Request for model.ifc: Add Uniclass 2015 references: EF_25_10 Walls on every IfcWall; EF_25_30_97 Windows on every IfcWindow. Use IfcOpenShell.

First a look at what the model holds.

```python
import ifcopenshell

model = ifcopenshell.open("model.ifc")
print(model.schema)
print("classifications:", [c.Name for c in model.by_type("IfcClassification")])
for ifc_class in ("IfcDoor", "IfcRoof", "IfcStair", "IfcWall", "IfcWindow"):
    print(ifc_class, len(model.by_type(ifc_class)))
```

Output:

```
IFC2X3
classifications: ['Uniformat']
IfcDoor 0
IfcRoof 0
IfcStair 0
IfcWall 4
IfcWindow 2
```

```python
import ifcopenshell
import ifcopenshell.api.classification

model = ifcopenshell.open("model.ifc")

# IFC2X3 requires Source and Edition and has no link from the project to the system.
system = model.create_entity("IfcClassification", Source="NBS", Edition="2015", Name="Uniclass 2015")

codes = {
    "IfcWall": ("EF_25_10", "Walls"),
    "IfcWindow": ("EF_25_30_97", "Windows"),
}
for ifc_class, (code, name) in codes.items():
    products = model.by_type(ifc_class)
    ifcopenshell.api.classification.add_reference(
        model, products=products, classification=system, identification=code, name=name
    )
    print(code, len(products))

model.write("model_edited.ifc")
```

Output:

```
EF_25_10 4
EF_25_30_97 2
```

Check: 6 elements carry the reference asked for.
